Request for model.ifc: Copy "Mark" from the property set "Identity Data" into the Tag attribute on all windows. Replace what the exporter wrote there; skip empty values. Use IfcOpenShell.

First a look at what the model holds.

```python
import ifcopenshell
import ifcopenshell.util.element

model = ifcopenshell.open("model.ifc")
print(model.schema)
windows = model.by_type("IfcWindow")
print(len(windows), "windows")
for e in windows[:8]:
    source = ifcopenshell.util.element.get_pset(e, "Identity Data", "Mark")
    target = e.Tag
    print(e.id(), repr(source), repr(target), sep=" | ")
```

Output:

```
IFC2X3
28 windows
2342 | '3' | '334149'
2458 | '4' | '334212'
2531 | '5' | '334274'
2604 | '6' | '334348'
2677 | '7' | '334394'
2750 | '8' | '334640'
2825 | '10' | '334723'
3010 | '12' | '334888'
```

```python
import ifcopenshell
import ifcopenshell.util.element

model = ifcopenshell.open("model.ifc")

count = 0
for e in model.by_type("IfcWindow"):
    value = ifcopenshell.util.element.get_pset(e, "Identity Data", "Mark")
    current = e.Tag
    if not value or not value.strip() or current == value:
        continue
    e.Tag = value
    count += 1

print(count, "windows updated")

model.write("model_v2.ifc")
```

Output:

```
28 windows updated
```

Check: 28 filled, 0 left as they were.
